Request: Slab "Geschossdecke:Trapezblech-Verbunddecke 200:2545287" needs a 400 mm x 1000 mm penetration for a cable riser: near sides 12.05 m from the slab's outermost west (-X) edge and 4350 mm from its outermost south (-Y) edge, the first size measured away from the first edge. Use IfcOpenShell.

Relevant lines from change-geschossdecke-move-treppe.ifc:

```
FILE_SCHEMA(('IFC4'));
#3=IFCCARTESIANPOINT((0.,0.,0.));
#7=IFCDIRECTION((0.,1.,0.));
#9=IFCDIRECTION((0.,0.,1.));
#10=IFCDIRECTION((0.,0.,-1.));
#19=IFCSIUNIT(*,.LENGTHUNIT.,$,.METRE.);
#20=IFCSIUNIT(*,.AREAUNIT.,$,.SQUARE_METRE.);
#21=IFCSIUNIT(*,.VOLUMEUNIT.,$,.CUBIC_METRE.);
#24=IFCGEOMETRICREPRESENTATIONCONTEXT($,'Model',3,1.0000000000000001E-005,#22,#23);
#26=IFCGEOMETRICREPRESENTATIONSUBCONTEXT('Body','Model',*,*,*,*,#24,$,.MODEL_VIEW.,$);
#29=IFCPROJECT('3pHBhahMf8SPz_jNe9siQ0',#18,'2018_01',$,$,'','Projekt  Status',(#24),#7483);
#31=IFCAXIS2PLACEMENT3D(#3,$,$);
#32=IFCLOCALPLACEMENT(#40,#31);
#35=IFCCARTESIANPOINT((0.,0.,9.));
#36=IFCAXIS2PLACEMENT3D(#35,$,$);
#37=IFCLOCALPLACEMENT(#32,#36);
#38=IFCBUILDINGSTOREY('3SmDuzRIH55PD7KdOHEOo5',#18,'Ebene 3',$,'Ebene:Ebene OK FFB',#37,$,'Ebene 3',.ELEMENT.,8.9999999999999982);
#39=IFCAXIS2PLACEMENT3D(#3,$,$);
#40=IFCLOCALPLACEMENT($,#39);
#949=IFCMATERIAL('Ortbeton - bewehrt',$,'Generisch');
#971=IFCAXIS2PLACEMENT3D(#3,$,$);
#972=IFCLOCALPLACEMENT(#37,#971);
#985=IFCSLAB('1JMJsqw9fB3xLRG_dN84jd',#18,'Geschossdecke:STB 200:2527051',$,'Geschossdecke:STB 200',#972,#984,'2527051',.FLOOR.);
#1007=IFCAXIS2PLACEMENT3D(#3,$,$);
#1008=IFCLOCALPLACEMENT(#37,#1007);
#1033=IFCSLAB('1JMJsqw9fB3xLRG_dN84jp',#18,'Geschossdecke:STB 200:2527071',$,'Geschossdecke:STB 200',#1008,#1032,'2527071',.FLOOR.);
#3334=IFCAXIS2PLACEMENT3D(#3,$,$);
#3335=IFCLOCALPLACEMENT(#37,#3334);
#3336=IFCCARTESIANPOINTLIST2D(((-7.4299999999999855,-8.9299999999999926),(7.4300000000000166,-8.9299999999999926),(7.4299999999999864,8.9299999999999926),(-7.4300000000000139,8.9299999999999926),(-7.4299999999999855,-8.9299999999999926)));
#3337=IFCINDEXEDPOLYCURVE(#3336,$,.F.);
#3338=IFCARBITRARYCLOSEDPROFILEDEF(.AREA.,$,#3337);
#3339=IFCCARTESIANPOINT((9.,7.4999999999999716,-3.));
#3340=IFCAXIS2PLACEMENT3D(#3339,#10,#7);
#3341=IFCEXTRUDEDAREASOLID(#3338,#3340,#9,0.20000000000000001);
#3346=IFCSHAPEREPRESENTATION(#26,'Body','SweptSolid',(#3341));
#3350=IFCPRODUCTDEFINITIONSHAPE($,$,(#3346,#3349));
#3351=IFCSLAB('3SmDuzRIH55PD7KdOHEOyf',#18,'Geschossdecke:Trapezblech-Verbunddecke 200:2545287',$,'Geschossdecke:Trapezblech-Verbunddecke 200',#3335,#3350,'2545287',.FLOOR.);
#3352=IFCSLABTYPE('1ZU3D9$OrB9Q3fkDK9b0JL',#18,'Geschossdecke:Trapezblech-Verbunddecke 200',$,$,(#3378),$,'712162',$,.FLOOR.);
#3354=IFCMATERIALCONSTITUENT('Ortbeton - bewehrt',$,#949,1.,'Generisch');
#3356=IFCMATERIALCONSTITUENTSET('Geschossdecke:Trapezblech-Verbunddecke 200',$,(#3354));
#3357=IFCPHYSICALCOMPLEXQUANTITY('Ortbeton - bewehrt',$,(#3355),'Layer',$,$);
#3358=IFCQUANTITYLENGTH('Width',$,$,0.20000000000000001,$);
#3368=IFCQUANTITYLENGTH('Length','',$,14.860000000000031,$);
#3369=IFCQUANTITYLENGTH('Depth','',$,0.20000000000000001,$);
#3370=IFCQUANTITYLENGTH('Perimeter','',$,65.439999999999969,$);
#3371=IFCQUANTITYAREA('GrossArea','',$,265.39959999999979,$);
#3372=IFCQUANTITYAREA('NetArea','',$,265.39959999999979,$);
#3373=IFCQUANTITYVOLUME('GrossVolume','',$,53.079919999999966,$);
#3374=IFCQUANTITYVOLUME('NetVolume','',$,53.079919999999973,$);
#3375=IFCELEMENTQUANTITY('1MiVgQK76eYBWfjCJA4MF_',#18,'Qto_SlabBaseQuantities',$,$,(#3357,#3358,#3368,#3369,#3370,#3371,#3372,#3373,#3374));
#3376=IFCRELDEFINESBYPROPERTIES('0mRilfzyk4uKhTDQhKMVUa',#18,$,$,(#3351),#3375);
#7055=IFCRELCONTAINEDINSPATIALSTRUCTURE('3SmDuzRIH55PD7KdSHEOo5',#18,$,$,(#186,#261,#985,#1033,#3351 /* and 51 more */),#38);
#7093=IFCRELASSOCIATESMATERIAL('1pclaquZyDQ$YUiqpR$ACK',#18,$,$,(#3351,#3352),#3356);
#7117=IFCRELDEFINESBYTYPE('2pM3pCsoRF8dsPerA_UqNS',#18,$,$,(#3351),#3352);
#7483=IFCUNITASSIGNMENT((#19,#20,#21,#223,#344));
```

```python
import numpy as np
import ifcopenshell
import ifcopenshell.api.feature
import ifcopenshell.api.geometry
import ifcopenshell.api.pset
import ifcopenshell.api.root
import ifcopenshell.geom
import ifcopenshell.util.element
import ifcopenshell.util.placement
import ifcopenshell.util.representation
import ifcopenshell.util.shape
import ifcopenshell.util.unit

model = ifcopenshell.open("change-geschossdecke-move-treppe.ifc")
unit_scale = ifcopenshell.util.unit.calculate_unit_scale(model)
area_scale = ifcopenshell.util.unit.calculate_unit_scale(model, "AREAUNIT")
volume_scale = ifcopenshell.util.unit.calculate_unit_scale(model, "VOLUMEUNIT")
settings = ifcopenshell.geom.settings()


def volume(element):
    """Net volume in cubic metres, openings subtracted."""
    shape = ifcopenshell.geom.create_shape(settings, element)
    return ifcopenshell.util.shape.get_volume(shape.geometry)


slab = model.by_id(3351)
before = volume(slab)

# Extent in the slab's own axes, in metres. The edges named are its -X and -Y sides.
slab_shape = ifcopenshell.geom.create_shape(settings, slab)
vertices = ifcopenshell.util.shape.get_vertices(slab_shape.geometry)
x_min, y_min, bottom = vertices.min(axis=0)
top = vertices[:, 2].max()

opening = ifcopenshell.api.root.create_entity(model, ifc_class="IfcOpeningElement", name="Cable riser opening", predefined_type="OPENING")
context = ifcopenshell.util.representation.get_context(model, "Model", "Body", "MODEL_VIEW")
width, depth = 0.4, 1
outline = [(0.0, 0.0), (width, 0.0), (width, depth), (0.0, depth), (0.0, 0.0)]
# Overshoot both faces by 50 mm so the cut is clean.
shape = ifcopenshell.api.geometry.add_slab_representation(
    model, context=context, depth=top - bottom + 0.1, polyline=outline
)
ifcopenshell.api.geometry.assign_representation(model, product=opening, representation=shape)

matrix = ifcopenshell.util.placement.get_local_placement(slab.ObjectPlacement)
matrix[:, 3] = matrix @ np.append(np.array([x_min + 12.05, y_min + 4.35, bottom - 0.05]) / unit_scale, 1.0)
ifcopenshell.api.geometry.edit_object_placement(model, product=opening, matrix=matrix, is_si=False)
ifcopenshell.api.feature.add_feature(model, feature=opening, element=slab)

after = volume(slab)

# Update the slab's stored quantities.
qto = model.by_id(ifcopenshell.util.element.get_pset(slab, "Qto_SlabBaseQuantities", should_inherit=False)["id"])
ifcopenshell.api.pset.edit_qto(model, qto=qto, properties={
    "NetArea": after / (top - bottom) / area_scale,
    "NetVolume": after / volume_scale,
})

print(f"slab volume {before:.3f} -> {after:.3f} m3")

model.write("change-geschossdecke-move-treppe_updated.ifc")
```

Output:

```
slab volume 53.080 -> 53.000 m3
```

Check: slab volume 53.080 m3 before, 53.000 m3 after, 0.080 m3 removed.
